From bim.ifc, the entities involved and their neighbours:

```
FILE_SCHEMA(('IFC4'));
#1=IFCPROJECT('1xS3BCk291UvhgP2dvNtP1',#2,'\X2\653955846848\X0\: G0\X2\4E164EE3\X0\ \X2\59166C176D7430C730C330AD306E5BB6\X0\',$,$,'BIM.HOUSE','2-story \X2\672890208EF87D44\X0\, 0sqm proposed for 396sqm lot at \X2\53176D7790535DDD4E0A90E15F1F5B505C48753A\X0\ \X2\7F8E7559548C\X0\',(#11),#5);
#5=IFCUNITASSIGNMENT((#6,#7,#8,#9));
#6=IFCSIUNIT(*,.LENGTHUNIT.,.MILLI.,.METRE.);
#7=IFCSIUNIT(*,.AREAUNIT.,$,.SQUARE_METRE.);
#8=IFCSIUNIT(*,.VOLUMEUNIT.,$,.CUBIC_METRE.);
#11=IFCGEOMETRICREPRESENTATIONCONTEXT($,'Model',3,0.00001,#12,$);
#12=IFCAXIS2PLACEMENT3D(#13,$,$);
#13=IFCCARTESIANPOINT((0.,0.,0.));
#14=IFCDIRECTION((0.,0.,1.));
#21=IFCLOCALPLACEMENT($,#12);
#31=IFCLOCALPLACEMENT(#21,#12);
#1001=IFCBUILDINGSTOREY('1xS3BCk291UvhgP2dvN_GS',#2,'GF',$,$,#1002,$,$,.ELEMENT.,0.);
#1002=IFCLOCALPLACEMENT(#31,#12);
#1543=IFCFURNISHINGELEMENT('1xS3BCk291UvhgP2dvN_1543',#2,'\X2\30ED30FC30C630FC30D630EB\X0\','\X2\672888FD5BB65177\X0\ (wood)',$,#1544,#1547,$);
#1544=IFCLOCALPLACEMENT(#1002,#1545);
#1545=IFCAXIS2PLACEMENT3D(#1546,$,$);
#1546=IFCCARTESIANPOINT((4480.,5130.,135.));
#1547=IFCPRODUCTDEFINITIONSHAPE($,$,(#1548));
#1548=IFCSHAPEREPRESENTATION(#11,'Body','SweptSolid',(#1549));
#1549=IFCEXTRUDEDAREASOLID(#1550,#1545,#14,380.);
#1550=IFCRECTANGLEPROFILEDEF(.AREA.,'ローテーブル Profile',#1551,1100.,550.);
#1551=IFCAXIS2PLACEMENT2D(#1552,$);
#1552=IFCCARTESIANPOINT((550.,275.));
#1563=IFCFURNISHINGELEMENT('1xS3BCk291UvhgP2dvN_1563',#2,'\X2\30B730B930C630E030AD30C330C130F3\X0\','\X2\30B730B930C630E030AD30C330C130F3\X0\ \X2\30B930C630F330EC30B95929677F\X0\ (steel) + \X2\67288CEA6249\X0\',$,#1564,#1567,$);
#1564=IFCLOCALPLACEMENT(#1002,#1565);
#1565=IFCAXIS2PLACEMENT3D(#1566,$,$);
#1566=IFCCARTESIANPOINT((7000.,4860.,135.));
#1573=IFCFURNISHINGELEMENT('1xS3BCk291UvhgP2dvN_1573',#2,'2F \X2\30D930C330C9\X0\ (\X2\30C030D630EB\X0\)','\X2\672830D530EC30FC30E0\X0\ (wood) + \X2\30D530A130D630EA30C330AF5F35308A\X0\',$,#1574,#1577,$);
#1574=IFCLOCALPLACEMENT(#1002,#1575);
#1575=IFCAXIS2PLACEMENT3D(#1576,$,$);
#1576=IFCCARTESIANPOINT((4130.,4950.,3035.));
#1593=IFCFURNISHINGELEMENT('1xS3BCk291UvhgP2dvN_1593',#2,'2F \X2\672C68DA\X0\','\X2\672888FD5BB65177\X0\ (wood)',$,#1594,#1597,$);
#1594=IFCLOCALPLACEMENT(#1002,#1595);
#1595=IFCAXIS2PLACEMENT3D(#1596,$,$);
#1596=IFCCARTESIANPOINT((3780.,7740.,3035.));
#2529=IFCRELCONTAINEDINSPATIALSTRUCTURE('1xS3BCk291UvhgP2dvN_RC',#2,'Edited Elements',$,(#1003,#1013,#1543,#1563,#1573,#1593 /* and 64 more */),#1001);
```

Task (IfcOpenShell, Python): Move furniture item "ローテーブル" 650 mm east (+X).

```python
import ifcopenshell
import ifcopenshell.api.geometry
import ifcopenshell.util.placement

model = ifcopenshell.open("bim.ifc")

item = model.by_guid("1xS3BCk291UvhgP2dvN_1543")
matrix = ifcopenshell.util.placement.get_local_placement(item.ObjectPlacement)
matrix[0, 3] += 650.0
ifcopenshell.api.geometry.edit_object_placement(model, product=item, matrix=matrix, is_si=False)

print(ifcopenshell.util.placement.get_local_placement(item.ObjectPlacement).round(3) + 0.0)

model.write("bim-out.ifc")
```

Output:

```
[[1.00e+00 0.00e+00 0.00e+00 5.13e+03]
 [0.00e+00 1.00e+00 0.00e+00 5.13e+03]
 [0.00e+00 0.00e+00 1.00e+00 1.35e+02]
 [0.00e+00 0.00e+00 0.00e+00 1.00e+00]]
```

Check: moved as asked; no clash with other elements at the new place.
